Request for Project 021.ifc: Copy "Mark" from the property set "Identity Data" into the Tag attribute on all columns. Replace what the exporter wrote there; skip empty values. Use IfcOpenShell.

First a look at what the model holds.

```python
import ifcopenshell
import ifcopenshell.util.element

model = ifcopenshell.open("Project 021.ifc")
print(model.schema)
columns = model.by_type("IfcColumn")
print(len(columns), "columns")
for e in columns[:8]:
    source = ifcopenshell.util.element.get_pset(e, "Identity Data", "Mark")
    target = e.Tag
    print(e.id(), repr(source), repr(target), sep=" | ")
```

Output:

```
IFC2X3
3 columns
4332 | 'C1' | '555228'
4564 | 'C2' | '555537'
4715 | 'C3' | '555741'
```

```python
import ifcopenshell
import ifcopenshell.util.element

model = ifcopenshell.open("Project 021.ifc")

count = 0
for e in model.by_type("IfcColumn"):
    value = ifcopenshell.util.element.get_pset(e, "Identity Data", "Mark")
    current = e.Tag
    if not value or not value.strip() or current == value:
        continue
    e.Tag = value
    count += 1

print(count, "columns updated")

model.write("Project 021_rev.ifc")
```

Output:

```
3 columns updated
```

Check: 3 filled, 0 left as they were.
